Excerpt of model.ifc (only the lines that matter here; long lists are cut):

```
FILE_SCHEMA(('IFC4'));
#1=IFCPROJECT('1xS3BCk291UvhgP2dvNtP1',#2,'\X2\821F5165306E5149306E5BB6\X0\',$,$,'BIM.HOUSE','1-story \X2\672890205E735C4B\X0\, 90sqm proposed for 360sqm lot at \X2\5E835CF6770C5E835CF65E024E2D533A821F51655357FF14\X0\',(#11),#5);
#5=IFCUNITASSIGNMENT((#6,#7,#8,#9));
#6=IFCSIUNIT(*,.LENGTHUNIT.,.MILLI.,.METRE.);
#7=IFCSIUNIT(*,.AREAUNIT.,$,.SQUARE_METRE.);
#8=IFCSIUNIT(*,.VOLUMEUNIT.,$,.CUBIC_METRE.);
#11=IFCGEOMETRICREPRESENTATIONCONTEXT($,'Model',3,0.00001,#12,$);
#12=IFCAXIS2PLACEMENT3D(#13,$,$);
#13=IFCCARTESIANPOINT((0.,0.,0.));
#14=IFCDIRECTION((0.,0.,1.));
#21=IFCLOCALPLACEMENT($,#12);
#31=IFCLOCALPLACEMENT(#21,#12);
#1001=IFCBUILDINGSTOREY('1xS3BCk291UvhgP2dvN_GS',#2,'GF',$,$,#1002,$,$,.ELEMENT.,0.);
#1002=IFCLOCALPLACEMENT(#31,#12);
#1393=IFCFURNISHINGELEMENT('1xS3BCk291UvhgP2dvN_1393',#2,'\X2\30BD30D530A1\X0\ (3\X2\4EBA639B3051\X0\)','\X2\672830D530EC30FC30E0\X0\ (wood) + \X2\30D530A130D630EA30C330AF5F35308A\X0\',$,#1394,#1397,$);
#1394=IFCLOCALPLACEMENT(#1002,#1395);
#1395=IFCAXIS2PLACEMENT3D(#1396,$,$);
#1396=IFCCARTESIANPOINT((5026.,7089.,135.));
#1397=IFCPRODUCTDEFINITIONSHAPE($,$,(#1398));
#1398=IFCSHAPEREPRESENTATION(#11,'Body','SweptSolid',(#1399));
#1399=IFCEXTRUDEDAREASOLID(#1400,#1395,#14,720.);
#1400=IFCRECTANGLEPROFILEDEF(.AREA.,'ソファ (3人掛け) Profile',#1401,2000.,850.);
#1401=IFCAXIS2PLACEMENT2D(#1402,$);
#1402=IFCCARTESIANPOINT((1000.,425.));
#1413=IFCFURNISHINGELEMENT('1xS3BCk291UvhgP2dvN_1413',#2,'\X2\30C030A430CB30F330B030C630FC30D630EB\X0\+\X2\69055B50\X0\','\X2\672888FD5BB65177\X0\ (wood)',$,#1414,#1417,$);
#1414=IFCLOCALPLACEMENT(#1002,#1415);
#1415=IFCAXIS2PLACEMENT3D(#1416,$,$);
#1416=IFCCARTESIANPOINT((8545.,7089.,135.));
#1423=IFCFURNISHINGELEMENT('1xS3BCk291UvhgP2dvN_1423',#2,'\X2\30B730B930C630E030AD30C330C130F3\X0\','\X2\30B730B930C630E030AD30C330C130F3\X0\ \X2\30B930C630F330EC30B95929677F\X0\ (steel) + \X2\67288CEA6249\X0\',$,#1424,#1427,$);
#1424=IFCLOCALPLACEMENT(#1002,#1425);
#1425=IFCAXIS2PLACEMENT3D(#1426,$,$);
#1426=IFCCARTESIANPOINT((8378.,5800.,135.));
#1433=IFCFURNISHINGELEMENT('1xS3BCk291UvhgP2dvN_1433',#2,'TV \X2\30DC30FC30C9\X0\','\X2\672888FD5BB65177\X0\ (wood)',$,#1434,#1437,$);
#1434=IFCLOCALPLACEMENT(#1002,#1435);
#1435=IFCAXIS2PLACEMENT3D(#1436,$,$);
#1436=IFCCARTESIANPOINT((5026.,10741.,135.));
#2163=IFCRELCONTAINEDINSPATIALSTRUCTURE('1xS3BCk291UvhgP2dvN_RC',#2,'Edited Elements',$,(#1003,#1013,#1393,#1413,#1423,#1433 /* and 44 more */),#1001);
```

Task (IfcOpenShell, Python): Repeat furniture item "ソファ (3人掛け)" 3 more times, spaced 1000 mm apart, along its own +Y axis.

```python
import ifcopenshell
import ifcopenshell.api.geometry
import ifcopenshell.api.root
import ifcopenshell.util.element
import ifcopenshell.util.placement
import ifcopenshell.util.unit

model = ifcopenshell.open("model.ifc")
unit_scale = ifcopenshell.util.unit.calculate_unit_scale(model)


def reuse_history(source, copy):
    """copy_class also copies each property set's owner history, people and application; keep the originals."""
    for rel in copy.IsDefinedBy:
        if rel.is_a("IfcRelDefinesByProperties") and (history := rel.RelatingPropertyDefinition.OwnerHistory):
            rel.RelatingPropertyDefinition.OwnerHistory = source.OwnerHistory
            ifcopenshell.util.element.remove_deep2(model, history)


source = model.by_guid("1xS3BCk291UvhgP2dvN_1393")
base = ifcopenshell.util.placement.get_local_placement(source.ObjectPlacement)
step = base[:3, 1] * 1 / unit_scale

for i in range(1, 4):
    copy = ifcopenshell.api.root.copy_class(model, product=source)
    copy.Representation = ifcopenshell.util.element.copy_deep(
        model, source.Representation, exclude=["IfcGeometricRepresentationContext", "IfcRepresentationMap"]
    )
    reuse_history(source, copy)
    matrix = base.copy()
    matrix[:3, 3] += i * step
    print("added at", matrix[:3, 3].round(3) + 0.0)
    ifcopenshell.api.geometry.edit_object_placement(model, product=copy, matrix=matrix, is_si=False)

model.write("model_rev.ifc")
```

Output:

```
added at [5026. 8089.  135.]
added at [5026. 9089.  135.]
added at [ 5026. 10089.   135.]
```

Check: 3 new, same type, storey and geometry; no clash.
